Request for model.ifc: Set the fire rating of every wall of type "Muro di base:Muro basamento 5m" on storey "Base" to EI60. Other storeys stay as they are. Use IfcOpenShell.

First a look at what the model holds.

```python
import ifcopenshell
import ifcopenshell.util.element

model = ifcopenshell.open("model.ifc")
print(model.schema)
storey = next(s for s in model.by_type("IfcBuildingStorey") if s.Name == "Base")
walls = [e for e in ifcopenshell.util.element.get_decomposition(storey) if e.is_a("IfcWall")]
seen = {}
for e in walls:
    element_type = ifcopenshell.util.element.get_type(e)
    key = (element_type.Name if element_type != e and element_type else None, ifcopenshell.util.element.get_pset(e, "Pset_WallCommon", "FireRating"))
    seen[key] = seen.get(key, 0) + 1
for (name, value), count in sorted(seen.items(), key=str):
    print(count, "x", name, "|", value)
```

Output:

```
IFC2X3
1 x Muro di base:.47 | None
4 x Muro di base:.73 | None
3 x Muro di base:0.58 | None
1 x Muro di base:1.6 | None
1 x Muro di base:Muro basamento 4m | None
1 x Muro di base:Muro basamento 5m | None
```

```python
import ifcopenshell
import ifcopenshell.api.pset
import ifcopenshell.util.element

model = ifcopenshell.open("model.ifc")

storey = next(s for s in model.by_type("IfcBuildingStorey") if s.Name == "Base")
walls = [e for e in ifcopenshell.util.element.get_decomposition(storey) if e.is_a("IfcWall")]

count = 0
for e in walls:
    element_type = ifcopenshell.util.element.get_type(e)
    if element_type in (None, e) or element_type.Name != "Muro di base:Muro basamento 5m":
        continue
    # add_pset returns the element's existing set when there is one.
    pset = ifcopenshell.api.pset.add_pset(model, product=e, name="Pset_WallCommon")
    ifcopenshell.api.pset.edit_pset(model, pset=pset, properties={"FireRating": "EI60"})
    count += 1

print(count, "walls updated")

model.write("model_edited.ifc")
```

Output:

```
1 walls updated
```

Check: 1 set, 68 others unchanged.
